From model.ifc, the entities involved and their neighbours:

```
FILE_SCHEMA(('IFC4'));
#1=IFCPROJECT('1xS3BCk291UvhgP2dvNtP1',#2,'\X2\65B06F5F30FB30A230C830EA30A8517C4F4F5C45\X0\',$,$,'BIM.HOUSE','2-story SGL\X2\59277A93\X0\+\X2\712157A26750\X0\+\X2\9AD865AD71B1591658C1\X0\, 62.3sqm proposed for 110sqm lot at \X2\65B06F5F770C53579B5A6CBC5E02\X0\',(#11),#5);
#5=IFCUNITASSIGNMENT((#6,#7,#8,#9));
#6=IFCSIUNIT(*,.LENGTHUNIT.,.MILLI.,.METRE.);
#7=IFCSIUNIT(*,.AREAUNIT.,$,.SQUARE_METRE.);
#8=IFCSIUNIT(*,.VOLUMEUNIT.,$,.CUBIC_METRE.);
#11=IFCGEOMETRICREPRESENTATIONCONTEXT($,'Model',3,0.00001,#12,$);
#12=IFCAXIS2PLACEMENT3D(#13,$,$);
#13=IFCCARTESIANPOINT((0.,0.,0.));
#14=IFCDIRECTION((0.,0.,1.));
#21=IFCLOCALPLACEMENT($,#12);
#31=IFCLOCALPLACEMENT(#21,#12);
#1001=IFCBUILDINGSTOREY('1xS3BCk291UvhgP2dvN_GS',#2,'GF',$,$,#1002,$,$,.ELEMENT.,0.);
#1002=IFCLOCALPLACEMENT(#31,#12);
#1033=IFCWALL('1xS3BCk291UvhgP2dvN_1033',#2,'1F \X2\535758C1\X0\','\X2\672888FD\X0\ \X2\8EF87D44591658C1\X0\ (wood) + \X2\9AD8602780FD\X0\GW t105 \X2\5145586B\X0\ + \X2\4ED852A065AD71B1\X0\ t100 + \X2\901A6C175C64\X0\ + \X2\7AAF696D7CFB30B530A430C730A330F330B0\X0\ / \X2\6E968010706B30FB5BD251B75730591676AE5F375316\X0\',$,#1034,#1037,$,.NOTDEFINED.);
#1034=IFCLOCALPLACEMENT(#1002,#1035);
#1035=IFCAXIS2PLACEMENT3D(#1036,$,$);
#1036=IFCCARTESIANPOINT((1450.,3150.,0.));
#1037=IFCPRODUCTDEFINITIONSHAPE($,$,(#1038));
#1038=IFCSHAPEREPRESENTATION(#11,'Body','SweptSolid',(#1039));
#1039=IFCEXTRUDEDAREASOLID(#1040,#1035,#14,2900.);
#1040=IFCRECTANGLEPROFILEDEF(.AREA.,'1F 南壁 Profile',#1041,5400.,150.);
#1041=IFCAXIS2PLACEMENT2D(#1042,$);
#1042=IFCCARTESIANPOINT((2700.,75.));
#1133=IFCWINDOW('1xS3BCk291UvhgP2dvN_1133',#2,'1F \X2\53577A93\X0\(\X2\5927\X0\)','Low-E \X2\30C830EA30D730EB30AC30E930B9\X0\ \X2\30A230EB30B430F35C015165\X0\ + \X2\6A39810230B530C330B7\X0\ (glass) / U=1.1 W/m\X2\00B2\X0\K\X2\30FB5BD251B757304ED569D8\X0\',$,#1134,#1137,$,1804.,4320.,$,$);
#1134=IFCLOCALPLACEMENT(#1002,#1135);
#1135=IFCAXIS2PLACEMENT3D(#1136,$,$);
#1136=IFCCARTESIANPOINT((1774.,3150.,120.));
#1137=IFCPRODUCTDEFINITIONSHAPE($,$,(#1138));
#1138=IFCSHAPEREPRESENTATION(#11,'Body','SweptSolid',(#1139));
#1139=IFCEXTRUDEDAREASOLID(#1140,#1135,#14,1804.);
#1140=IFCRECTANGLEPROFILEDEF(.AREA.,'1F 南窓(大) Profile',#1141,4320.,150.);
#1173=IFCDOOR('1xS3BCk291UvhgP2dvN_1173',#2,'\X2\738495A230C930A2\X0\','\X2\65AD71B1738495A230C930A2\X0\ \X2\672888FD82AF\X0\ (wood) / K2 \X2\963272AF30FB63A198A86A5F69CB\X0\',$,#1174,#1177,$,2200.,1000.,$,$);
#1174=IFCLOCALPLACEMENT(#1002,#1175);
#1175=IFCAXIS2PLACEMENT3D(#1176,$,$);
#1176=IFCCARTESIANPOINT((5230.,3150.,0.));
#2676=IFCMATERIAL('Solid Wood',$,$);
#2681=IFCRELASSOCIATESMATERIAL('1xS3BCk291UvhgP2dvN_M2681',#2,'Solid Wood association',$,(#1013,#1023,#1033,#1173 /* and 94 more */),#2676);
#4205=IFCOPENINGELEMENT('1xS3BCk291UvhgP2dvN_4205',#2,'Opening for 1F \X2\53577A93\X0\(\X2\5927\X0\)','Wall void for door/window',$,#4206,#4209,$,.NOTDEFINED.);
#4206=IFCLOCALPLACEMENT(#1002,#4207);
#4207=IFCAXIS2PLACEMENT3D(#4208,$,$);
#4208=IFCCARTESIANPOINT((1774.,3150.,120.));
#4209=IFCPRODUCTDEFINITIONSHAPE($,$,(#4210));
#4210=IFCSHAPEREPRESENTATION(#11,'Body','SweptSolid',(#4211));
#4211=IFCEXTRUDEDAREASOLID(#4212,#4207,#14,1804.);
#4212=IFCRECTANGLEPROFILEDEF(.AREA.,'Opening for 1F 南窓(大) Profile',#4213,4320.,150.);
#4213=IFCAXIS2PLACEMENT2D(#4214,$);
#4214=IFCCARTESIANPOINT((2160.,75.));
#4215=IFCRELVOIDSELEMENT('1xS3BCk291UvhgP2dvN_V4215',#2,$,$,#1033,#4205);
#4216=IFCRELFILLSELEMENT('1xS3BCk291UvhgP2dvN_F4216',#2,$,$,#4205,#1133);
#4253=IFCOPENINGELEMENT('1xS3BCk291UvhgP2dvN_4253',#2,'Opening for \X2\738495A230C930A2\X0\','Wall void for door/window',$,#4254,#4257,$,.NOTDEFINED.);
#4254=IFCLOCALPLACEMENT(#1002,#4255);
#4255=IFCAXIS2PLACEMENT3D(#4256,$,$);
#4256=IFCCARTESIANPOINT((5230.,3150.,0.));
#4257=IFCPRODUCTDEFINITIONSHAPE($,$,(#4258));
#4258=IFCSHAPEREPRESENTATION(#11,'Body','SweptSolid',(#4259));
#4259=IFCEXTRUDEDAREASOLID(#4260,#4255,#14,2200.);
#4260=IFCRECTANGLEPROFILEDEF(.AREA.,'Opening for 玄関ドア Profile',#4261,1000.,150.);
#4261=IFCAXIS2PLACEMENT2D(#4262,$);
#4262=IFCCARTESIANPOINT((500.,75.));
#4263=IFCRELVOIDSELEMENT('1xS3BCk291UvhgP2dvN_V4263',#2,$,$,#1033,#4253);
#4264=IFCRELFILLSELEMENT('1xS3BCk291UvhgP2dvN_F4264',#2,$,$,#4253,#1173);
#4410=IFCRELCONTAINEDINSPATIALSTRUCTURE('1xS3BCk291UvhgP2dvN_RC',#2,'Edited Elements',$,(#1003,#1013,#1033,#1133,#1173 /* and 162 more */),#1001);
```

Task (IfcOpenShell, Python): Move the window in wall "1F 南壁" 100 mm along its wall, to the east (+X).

```python
import ifcopenshell
import ifcopenshell.api.geometry
import ifcopenshell.util.placement
import ifcopenshell.util.unit

model = ifcopenshell.open("model.ifc")
unit_scale = ifcopenshell.util.unit.calculate_unit_scale(model)

window = model.by_guid("1xS3BCk291UvhgP2dvN_1133")
opening = window.FillsVoids[0].RelatingOpeningElement
wall = opening.VoidsElements[0].RelatingBuildingElement

wall_matrix = ifcopenshell.util.placement.get_local_placement(wall.ObjectPlacement)
shift = wall_matrix[:3, 0] * 0.1 / unit_scale
before = ifcopenshell.util.placement.get_local_placement(window.ObjectPlacement)[:3, 3].copy()

# The window is not placed relative to its opening, so move both.
for product in (opening, window):
    matrix = ifcopenshell.util.placement.get_local_placement(product.ObjectPlacement)
    matrix[:3, 3] += shift
    ifcopenshell.api.geometry.edit_object_placement(model, product=product, matrix=matrix, is_si=False)

after = ifcopenshell.util.placement.get_local_placement(window.ObjectPlacement)[:3, 3]
print("window moved by", (after - before).round(3) + 0.0)

model.write("model_v2.ifc")
```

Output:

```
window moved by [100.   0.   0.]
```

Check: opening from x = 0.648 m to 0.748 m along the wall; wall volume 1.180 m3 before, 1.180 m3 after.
